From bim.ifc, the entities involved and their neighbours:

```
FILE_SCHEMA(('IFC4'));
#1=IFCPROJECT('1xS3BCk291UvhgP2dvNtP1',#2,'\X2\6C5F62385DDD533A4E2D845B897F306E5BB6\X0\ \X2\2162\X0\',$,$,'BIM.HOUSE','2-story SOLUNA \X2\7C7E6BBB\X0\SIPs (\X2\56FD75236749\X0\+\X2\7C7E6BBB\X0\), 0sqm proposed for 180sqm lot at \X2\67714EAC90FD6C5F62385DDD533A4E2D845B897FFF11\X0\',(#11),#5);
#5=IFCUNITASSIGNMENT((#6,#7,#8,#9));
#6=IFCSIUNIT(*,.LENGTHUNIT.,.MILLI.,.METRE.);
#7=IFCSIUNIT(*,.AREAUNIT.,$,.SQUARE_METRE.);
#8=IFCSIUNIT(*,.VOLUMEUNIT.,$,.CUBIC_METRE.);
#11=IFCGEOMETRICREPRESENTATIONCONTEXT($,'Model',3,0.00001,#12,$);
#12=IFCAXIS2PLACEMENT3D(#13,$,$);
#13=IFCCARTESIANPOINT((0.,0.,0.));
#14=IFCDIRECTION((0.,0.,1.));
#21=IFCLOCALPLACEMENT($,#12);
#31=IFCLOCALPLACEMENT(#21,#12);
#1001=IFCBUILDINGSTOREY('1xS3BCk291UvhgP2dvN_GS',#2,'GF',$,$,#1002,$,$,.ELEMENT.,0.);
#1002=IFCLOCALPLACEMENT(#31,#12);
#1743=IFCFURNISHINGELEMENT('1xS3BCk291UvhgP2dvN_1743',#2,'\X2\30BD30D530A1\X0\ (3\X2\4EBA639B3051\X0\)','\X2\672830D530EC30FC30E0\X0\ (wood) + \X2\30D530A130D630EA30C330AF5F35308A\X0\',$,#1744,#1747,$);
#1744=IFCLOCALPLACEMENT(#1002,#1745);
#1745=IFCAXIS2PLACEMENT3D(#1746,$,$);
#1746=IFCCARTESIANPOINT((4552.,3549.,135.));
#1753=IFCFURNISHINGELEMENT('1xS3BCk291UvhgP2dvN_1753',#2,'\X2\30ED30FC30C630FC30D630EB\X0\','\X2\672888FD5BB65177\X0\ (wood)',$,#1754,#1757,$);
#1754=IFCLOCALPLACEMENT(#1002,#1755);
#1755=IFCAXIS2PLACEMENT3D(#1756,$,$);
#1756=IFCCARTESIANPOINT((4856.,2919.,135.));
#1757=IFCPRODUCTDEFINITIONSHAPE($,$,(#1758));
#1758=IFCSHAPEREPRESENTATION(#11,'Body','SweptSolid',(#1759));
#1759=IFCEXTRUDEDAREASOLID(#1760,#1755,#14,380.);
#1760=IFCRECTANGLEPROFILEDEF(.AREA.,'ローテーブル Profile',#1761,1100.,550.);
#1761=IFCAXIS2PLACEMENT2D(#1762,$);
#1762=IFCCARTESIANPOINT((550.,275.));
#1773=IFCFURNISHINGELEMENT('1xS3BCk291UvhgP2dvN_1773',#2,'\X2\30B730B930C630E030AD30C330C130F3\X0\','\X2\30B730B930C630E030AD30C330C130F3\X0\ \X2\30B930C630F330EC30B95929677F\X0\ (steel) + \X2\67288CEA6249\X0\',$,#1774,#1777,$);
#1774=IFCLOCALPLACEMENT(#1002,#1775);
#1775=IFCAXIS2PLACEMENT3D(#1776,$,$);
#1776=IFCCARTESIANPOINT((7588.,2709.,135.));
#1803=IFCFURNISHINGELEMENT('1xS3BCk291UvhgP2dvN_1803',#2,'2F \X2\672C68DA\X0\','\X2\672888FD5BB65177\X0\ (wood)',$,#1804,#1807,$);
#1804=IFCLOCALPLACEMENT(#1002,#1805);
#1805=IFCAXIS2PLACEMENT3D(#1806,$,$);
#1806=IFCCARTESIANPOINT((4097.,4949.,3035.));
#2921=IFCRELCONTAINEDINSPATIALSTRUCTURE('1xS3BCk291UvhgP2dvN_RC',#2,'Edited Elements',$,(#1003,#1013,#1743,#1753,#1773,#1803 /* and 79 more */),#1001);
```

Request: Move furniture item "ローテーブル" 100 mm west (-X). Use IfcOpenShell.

```python
import ifcopenshell
import ifcopenshell.api.geometry
import ifcopenshell.util.placement
import ifcopenshell.util.unit

model = ifcopenshell.open("bim.ifc")
unit_scale = ifcopenshell.util.unit.calculate_unit_scale(model)

item = model.by_id(1753)
matrix = ifcopenshell.util.placement.get_local_placement(item.ObjectPlacement)
matrix[0, 3] -= 0.1 / unit_scale
ifcopenshell.api.geometry.edit_object_placement(model, product=item, matrix=matrix, is_si=False)

print(ifcopenshell.util.placement.get_local_placement(item.ObjectPlacement).round(3) + 0.0)

model.write("bim_rev.ifc")
```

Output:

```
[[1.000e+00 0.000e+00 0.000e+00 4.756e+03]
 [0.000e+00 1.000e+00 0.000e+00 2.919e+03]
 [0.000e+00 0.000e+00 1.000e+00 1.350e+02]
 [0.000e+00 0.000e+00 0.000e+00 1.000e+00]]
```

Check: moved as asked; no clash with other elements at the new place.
